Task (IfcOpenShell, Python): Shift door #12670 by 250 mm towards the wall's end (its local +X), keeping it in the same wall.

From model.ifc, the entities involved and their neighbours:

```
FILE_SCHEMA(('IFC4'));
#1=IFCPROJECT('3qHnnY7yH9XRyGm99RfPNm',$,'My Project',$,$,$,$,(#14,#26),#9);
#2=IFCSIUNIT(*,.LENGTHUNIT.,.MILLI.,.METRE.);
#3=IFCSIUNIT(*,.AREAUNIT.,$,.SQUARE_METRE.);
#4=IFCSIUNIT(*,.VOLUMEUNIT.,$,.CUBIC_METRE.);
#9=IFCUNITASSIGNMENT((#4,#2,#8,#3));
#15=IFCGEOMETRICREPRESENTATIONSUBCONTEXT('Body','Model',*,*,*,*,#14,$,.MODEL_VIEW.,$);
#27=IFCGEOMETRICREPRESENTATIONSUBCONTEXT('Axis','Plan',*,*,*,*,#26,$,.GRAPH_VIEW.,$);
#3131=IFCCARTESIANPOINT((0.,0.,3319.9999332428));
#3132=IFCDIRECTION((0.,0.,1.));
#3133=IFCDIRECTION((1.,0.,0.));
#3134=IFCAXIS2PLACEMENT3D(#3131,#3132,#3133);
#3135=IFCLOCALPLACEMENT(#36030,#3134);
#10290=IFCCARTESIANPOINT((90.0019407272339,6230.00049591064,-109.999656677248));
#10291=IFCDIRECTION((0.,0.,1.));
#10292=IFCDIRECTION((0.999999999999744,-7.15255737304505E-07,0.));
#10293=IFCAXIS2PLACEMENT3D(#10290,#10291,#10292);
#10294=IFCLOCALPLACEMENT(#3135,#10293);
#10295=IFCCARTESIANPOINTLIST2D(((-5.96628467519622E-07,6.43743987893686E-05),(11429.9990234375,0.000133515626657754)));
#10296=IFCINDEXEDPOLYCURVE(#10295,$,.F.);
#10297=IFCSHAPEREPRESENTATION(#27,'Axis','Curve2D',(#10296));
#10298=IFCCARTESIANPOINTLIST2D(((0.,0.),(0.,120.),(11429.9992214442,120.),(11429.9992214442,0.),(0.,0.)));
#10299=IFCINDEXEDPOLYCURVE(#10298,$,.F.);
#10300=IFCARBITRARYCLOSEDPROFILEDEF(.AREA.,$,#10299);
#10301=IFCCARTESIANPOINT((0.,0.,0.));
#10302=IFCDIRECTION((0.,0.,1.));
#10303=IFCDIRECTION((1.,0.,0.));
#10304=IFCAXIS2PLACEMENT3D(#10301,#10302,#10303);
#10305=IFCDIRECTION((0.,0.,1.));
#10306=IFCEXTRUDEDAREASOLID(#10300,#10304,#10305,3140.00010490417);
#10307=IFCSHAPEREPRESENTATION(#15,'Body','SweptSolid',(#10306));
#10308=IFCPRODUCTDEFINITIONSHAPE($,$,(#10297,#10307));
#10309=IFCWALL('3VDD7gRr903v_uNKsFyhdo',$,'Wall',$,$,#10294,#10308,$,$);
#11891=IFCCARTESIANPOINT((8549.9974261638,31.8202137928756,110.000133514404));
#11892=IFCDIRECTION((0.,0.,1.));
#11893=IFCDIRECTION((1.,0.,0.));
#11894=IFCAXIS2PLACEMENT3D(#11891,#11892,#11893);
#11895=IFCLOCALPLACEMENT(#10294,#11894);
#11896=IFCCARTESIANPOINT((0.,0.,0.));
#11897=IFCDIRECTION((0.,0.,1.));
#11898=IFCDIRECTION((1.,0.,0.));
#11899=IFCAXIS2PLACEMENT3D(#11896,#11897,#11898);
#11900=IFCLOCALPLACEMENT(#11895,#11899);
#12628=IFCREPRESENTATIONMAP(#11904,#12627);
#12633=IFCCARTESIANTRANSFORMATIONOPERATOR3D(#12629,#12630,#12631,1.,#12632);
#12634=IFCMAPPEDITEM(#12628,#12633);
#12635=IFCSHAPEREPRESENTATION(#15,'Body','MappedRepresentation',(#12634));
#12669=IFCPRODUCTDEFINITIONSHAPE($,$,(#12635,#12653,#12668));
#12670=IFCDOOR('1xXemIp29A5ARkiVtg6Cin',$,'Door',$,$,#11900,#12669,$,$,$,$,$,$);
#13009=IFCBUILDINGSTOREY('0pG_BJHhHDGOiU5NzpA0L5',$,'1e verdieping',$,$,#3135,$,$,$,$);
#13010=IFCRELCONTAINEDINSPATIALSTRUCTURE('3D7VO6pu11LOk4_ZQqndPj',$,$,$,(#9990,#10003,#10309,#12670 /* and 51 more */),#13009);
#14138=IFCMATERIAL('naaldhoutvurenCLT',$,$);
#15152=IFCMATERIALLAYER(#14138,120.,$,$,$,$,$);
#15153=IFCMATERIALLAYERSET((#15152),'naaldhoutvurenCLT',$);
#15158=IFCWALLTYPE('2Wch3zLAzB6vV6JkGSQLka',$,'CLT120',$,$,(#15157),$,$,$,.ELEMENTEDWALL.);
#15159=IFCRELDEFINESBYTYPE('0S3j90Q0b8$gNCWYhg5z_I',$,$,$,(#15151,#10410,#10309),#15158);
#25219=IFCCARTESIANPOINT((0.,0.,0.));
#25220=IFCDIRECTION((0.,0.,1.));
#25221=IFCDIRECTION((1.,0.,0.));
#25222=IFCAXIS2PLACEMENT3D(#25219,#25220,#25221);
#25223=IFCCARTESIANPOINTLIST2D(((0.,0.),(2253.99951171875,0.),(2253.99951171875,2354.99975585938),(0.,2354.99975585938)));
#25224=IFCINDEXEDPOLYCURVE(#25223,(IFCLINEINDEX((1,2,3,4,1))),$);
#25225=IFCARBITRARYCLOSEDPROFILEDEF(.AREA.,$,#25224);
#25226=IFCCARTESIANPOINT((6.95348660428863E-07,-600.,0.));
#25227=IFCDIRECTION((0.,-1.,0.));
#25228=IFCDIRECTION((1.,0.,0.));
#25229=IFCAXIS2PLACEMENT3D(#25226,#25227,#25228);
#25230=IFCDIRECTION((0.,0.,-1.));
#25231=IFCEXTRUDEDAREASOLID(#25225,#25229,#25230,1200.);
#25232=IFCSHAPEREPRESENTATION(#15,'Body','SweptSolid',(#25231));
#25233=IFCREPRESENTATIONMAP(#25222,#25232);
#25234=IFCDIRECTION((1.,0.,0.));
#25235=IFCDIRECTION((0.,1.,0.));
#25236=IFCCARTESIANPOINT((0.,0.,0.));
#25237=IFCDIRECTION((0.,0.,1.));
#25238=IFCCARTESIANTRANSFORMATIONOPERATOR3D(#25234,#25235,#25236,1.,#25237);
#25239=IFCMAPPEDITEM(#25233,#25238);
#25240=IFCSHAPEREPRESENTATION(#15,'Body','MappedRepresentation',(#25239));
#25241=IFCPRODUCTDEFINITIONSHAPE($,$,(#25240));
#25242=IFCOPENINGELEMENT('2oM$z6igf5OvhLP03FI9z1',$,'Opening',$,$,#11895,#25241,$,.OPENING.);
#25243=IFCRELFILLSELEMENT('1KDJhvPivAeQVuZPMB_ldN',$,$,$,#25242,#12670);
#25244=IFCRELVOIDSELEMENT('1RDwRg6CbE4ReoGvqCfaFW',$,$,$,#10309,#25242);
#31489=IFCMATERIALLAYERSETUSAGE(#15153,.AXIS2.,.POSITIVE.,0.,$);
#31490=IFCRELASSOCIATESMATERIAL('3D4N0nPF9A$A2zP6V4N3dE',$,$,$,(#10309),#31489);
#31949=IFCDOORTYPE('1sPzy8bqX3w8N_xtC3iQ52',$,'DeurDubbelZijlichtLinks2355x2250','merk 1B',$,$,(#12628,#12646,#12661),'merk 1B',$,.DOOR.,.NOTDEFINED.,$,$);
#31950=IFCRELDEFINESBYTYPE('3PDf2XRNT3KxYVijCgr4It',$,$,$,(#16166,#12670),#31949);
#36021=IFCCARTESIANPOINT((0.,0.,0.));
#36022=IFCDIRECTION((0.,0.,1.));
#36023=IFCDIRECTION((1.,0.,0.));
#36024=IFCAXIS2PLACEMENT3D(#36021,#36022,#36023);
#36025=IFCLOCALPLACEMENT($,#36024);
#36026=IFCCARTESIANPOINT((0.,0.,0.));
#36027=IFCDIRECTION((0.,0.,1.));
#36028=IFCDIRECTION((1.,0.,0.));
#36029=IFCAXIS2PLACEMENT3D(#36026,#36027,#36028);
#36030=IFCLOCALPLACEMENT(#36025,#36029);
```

```python
import ifcopenshell
import ifcopenshell.api.geometry
import ifcopenshell.util.placement

model = ifcopenshell.open("model.ifc")

door = model.by_id(12670)
opening = door.FillsVoids[0].RelatingOpeningElement
wall = opening.VoidsElements[0].RelatingBuildingElement

wall_matrix = ifcopenshell.util.placement.get_local_placement(wall.ObjectPlacement)
shift = wall_matrix[:3, 0] * 250.0
before = ifcopenshell.util.placement.get_local_placement(door.ObjectPlacement)[:3, 3].copy()

# The door is placed relative to its opening, so it follows when the opening moves.
matrix = ifcopenshell.util.placement.get_local_placement(opening.ObjectPlacement)
matrix[:3, 3] += shift
ifcopenshell.api.geometry.edit_object_placement(
    model, product=opening, matrix=matrix, is_si=False, should_transform_children=True
)

after = ifcopenshell.util.placement.get_local_placement(door.ObjectPlacement)[:3, 3]
print("door moved by", (after - before).round(3) + 0.0)

model.write("model_updated.ifc")
```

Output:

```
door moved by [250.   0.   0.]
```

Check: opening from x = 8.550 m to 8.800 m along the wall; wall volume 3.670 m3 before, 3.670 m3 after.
